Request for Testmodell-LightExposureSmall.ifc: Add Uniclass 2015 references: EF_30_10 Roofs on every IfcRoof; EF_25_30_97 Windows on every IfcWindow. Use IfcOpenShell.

First a look at what the model holds.

```python
import ifcopenshell

model = ifcopenshell.open("Testmodell-LightExposureSmall.ifc")
print(model.schema)
print("classifications:", [c.Name for c in model.by_type("IfcClassification")])
for ifc_class in ("IfcDoor", "IfcRoof", "IfcStair", "IfcWall", "IfcWindow"):
    print(ifc_class, len(model.by_type(ifc_class)))
```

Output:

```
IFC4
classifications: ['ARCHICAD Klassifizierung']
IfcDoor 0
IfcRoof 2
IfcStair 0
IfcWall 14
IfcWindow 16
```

```python
import ifcopenshell
import ifcopenshell.api.classification

model = ifcopenshell.open("Testmodell-LightExposureSmall.ifc")

system = ifcopenshell.api.classification.add_classification(model, classification="Uniclass 2015")

codes = {
    "IfcRoof": ("EF_30_10", "Roofs"),
    "IfcWindow": ("EF_25_30_97", "Windows"),
}
for ifc_class, (code, name) in codes.items():
    products = model.by_type(ifc_class)
    ifcopenshell.api.classification.add_reference(
        model, products=products, classification=system, identification=code, name=name
    )
    print(code, len(products))

model.write("Testmodell-LightExposureSmall_rev.ifc")
```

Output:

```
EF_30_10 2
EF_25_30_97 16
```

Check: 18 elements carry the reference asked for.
